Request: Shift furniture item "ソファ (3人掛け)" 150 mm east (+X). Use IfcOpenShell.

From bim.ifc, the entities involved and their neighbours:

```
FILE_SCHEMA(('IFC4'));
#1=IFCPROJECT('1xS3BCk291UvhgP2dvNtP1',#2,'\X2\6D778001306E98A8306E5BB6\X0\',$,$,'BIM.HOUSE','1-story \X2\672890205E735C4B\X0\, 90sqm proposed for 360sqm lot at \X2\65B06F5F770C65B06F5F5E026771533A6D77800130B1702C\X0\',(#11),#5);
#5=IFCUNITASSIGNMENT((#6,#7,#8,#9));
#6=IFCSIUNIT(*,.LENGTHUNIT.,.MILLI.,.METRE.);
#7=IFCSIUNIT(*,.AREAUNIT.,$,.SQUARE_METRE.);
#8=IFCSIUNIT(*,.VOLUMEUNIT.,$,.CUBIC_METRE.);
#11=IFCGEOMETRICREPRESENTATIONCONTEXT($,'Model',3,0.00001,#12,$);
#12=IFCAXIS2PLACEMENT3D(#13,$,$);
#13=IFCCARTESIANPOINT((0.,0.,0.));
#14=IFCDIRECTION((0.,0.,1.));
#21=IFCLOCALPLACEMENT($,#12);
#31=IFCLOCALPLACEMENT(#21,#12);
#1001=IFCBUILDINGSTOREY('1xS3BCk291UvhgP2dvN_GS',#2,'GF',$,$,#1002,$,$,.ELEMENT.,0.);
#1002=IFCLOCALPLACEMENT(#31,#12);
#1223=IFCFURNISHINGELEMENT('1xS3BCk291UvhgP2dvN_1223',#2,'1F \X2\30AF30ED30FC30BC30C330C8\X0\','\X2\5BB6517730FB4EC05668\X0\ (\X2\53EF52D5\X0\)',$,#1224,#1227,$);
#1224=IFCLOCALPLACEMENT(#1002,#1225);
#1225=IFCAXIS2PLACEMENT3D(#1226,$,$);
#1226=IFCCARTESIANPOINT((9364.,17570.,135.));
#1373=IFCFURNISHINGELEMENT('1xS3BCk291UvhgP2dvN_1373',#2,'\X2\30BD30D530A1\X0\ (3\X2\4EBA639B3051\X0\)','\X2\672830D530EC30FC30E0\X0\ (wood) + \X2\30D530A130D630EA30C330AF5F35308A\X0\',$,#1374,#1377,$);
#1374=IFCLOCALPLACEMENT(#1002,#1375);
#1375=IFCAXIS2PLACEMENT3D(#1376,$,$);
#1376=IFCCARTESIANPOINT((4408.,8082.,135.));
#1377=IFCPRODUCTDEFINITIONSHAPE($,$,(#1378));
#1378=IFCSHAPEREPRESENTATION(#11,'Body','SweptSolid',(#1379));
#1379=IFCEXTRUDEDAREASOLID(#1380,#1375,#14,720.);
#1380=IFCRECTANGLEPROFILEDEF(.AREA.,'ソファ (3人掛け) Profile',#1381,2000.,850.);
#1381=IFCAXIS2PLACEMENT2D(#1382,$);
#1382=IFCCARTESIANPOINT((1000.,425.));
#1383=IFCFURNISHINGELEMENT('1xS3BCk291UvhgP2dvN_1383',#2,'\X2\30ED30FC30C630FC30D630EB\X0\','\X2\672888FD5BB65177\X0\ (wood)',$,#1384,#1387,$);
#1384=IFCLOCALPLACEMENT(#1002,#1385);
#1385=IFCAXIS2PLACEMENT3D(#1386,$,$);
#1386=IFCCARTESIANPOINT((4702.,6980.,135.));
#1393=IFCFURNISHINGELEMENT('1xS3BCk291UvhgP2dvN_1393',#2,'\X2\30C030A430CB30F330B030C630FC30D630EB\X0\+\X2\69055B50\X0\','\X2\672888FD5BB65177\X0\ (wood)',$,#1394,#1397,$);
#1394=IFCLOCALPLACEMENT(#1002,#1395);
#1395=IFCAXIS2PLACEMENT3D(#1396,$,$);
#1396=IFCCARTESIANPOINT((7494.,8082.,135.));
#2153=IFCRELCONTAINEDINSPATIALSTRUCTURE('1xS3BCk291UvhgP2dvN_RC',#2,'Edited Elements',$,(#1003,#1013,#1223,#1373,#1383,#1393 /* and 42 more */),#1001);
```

```python
import ifcopenshell
import ifcopenshell.api.geometry
import ifcopenshell.util.placement
import ifcopenshell.util.unit

model = ifcopenshell.open("bim.ifc")
unit_scale = ifcopenshell.util.unit.calculate_unit_scale(model)

item = model.by_id(1373)
matrix = ifcopenshell.util.placement.get_local_placement(item.ObjectPlacement)
matrix[0, 3] += 0.15 / unit_scale
ifcopenshell.api.geometry.edit_object_placement(model, product=item, matrix=matrix, is_si=False)

print(ifcopenshell.util.placement.get_local_placement(item.ObjectPlacement).round(3) + 0.0)

model.write("bim_edited.ifc")
```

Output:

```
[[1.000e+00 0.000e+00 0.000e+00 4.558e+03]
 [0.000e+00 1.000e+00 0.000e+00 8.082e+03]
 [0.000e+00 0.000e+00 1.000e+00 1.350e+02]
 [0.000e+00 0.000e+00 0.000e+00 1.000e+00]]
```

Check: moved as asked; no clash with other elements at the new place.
